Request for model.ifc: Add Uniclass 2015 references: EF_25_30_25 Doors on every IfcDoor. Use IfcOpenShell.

First a look at what the model holds.

```python
import ifcopenshell

model = ifcopenshell.open("model.ifc")
print(model.schema)
print("classifications:", [c.Name for c in model.by_type("IfcClassification")])
for ifc_class in ("IfcDoor", "IfcRoof", "IfcStair", "IfcWall", "IfcWindow"):
    print(ifc_class, len(model.by_type(ifc_class)))
```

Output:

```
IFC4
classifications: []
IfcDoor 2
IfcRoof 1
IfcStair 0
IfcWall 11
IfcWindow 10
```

```python
import ifcopenshell
import ifcopenshell.api.classification

model = ifcopenshell.open("model.ifc")

system = ifcopenshell.api.classification.add_classification(model, classification="Uniclass 2015")

codes = {
    "IfcDoor": ("EF_25_30_25", "Doors"),
}
for ifc_class, (code, name) in codes.items():
    products = model.by_type(ifc_class)
    ifcopenshell.api.classification.add_reference(
        model, products=products, classification=system, identification=code, name=name
    )
    print(code, len(products))

model.write("model-out.ifc")
```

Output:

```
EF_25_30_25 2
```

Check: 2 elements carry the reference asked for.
